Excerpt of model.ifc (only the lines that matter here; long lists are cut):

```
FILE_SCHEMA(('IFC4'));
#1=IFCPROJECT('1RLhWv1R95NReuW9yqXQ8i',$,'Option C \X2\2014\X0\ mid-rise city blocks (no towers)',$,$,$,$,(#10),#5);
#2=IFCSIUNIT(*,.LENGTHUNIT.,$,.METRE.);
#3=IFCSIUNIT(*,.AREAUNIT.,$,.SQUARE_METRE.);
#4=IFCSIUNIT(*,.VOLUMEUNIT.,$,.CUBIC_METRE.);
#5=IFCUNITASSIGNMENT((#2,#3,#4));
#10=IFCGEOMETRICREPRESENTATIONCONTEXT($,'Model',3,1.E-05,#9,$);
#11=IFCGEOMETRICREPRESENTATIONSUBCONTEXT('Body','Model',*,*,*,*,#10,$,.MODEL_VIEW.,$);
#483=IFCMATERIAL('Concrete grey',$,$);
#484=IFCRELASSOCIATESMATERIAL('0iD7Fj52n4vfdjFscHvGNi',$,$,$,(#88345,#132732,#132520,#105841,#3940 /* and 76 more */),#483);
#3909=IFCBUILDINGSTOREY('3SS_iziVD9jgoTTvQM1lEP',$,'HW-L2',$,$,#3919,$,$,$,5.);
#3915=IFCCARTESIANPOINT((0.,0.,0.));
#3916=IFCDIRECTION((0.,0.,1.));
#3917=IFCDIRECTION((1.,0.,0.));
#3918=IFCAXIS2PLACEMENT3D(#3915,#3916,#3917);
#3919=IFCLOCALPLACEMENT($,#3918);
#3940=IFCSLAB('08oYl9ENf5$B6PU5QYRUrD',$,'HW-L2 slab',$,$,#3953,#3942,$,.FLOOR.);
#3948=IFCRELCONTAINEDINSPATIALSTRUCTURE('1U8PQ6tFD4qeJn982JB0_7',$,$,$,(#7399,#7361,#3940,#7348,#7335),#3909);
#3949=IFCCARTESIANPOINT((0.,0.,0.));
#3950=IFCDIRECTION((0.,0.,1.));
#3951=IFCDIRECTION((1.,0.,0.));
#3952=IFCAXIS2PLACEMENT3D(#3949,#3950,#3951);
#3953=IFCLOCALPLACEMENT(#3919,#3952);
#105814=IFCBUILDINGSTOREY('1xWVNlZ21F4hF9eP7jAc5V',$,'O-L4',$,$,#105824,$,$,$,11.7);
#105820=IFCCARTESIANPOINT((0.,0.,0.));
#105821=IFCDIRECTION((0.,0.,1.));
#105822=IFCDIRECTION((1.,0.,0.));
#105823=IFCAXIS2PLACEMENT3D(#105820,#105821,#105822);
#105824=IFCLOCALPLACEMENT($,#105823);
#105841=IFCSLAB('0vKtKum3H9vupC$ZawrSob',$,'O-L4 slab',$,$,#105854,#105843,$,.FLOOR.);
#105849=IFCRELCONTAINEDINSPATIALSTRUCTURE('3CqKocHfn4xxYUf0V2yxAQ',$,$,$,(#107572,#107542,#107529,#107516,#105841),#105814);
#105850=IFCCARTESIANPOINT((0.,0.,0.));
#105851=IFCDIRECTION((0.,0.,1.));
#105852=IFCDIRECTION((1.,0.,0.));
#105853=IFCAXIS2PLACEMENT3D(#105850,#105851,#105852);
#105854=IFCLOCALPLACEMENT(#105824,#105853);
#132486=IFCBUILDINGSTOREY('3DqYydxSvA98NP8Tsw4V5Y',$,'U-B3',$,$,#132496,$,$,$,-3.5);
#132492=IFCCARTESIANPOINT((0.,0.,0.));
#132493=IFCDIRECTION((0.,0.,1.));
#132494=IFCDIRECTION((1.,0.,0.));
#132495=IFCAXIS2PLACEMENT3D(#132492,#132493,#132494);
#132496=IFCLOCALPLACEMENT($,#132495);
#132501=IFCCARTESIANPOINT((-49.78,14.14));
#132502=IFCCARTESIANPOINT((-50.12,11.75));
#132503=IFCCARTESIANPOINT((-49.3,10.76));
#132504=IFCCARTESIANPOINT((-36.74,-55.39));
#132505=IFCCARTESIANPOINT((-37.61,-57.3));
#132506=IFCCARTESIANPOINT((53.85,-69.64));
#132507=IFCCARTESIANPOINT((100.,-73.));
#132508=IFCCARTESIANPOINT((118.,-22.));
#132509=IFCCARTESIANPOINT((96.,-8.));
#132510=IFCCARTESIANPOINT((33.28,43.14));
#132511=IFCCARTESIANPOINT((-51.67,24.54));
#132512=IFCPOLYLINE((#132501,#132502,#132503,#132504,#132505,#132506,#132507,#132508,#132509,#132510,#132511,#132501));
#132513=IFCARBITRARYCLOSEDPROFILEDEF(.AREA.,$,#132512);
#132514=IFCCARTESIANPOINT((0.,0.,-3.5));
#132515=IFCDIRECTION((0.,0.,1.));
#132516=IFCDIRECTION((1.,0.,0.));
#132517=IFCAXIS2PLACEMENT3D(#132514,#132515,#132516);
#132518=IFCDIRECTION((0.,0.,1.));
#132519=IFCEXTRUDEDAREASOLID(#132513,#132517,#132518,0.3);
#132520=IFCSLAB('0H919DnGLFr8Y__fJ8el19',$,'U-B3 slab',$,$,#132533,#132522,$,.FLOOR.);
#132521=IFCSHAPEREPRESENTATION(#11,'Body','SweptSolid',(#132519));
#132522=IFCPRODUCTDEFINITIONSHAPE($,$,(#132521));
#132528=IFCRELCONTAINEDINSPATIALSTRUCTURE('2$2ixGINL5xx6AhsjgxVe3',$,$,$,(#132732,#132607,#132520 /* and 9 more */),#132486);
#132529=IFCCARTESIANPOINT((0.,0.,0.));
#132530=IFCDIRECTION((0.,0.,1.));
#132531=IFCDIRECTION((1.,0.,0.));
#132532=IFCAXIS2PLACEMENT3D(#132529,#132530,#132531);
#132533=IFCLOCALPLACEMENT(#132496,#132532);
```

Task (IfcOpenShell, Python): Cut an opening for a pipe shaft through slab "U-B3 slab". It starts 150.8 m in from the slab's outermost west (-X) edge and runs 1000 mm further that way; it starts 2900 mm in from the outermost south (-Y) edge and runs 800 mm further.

```python
import numpy as np
import ifcopenshell
import ifcopenshell.api.feature
import ifcopenshell.api.geometry
import ifcopenshell.api.root
import ifcopenshell.geom
import ifcopenshell.util.placement
import ifcopenshell.util.representation
import ifcopenshell.util.shape
import ifcopenshell.util.unit

model = ifcopenshell.open("model.ifc")
unit_scale = ifcopenshell.util.unit.calculate_unit_scale(model)
settings = ifcopenshell.geom.settings()


def volume(element):
    """Net volume in cubic metres, openings subtracted."""
    shape = ifcopenshell.geom.create_shape(settings, element)
    return ifcopenshell.util.shape.get_volume(shape.geometry)


slab = model.by_guid("0H919DnGLFr8Y__fJ8el19")
before = volume(slab)

# Extent in the slab's own axes, in metres. The edges named are its -X and -Y sides.
slab_shape = ifcopenshell.geom.create_shape(settings, slab)
vertices = ifcopenshell.util.shape.get_vertices(slab_shape.geometry)
x_min, y_min, bottom = vertices.min(axis=0)
top = vertices[:, 2].max()

opening = ifcopenshell.api.root.create_entity(model, ifc_class="IfcOpeningElement", name="Pipe shaft opening", predefined_type="OPENING")
context = ifcopenshell.util.representation.get_context(model, "Model", "Body", "MODEL_VIEW")
width, depth = 1, 0.8
outline = [(0.0, 0.0), (width, 0.0), (width, depth), (0.0, depth), (0.0, 0.0)]
# Overshoot both faces by 50 mm so the cut is clean.
shape = ifcopenshell.api.geometry.add_slab_representation(
    model, context=context, depth=top - bottom + 0.1, polyline=outline
)
ifcopenshell.api.geometry.assign_representation(model, product=opening, representation=shape)

matrix = ifcopenshell.util.placement.get_local_placement(slab.ObjectPlacement)
matrix[:, 3] = matrix @ np.append(np.array([x_min + 150.8, y_min + 2.9, bottom - 0.05]) / unit_scale, 1.0)
ifcopenshell.api.geometry.edit_object_placement(model, product=opening, matrix=matrix, is_si=False)
ifcopenshell.api.feature.add_feature(model, feature=opening, element=slab)

after = volume(slab)

print(f"slab volume {before:.3f} -> {after:.3f} m3")

model.write("model_rev.ifc")
```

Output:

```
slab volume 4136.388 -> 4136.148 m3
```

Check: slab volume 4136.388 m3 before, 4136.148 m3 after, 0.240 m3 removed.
